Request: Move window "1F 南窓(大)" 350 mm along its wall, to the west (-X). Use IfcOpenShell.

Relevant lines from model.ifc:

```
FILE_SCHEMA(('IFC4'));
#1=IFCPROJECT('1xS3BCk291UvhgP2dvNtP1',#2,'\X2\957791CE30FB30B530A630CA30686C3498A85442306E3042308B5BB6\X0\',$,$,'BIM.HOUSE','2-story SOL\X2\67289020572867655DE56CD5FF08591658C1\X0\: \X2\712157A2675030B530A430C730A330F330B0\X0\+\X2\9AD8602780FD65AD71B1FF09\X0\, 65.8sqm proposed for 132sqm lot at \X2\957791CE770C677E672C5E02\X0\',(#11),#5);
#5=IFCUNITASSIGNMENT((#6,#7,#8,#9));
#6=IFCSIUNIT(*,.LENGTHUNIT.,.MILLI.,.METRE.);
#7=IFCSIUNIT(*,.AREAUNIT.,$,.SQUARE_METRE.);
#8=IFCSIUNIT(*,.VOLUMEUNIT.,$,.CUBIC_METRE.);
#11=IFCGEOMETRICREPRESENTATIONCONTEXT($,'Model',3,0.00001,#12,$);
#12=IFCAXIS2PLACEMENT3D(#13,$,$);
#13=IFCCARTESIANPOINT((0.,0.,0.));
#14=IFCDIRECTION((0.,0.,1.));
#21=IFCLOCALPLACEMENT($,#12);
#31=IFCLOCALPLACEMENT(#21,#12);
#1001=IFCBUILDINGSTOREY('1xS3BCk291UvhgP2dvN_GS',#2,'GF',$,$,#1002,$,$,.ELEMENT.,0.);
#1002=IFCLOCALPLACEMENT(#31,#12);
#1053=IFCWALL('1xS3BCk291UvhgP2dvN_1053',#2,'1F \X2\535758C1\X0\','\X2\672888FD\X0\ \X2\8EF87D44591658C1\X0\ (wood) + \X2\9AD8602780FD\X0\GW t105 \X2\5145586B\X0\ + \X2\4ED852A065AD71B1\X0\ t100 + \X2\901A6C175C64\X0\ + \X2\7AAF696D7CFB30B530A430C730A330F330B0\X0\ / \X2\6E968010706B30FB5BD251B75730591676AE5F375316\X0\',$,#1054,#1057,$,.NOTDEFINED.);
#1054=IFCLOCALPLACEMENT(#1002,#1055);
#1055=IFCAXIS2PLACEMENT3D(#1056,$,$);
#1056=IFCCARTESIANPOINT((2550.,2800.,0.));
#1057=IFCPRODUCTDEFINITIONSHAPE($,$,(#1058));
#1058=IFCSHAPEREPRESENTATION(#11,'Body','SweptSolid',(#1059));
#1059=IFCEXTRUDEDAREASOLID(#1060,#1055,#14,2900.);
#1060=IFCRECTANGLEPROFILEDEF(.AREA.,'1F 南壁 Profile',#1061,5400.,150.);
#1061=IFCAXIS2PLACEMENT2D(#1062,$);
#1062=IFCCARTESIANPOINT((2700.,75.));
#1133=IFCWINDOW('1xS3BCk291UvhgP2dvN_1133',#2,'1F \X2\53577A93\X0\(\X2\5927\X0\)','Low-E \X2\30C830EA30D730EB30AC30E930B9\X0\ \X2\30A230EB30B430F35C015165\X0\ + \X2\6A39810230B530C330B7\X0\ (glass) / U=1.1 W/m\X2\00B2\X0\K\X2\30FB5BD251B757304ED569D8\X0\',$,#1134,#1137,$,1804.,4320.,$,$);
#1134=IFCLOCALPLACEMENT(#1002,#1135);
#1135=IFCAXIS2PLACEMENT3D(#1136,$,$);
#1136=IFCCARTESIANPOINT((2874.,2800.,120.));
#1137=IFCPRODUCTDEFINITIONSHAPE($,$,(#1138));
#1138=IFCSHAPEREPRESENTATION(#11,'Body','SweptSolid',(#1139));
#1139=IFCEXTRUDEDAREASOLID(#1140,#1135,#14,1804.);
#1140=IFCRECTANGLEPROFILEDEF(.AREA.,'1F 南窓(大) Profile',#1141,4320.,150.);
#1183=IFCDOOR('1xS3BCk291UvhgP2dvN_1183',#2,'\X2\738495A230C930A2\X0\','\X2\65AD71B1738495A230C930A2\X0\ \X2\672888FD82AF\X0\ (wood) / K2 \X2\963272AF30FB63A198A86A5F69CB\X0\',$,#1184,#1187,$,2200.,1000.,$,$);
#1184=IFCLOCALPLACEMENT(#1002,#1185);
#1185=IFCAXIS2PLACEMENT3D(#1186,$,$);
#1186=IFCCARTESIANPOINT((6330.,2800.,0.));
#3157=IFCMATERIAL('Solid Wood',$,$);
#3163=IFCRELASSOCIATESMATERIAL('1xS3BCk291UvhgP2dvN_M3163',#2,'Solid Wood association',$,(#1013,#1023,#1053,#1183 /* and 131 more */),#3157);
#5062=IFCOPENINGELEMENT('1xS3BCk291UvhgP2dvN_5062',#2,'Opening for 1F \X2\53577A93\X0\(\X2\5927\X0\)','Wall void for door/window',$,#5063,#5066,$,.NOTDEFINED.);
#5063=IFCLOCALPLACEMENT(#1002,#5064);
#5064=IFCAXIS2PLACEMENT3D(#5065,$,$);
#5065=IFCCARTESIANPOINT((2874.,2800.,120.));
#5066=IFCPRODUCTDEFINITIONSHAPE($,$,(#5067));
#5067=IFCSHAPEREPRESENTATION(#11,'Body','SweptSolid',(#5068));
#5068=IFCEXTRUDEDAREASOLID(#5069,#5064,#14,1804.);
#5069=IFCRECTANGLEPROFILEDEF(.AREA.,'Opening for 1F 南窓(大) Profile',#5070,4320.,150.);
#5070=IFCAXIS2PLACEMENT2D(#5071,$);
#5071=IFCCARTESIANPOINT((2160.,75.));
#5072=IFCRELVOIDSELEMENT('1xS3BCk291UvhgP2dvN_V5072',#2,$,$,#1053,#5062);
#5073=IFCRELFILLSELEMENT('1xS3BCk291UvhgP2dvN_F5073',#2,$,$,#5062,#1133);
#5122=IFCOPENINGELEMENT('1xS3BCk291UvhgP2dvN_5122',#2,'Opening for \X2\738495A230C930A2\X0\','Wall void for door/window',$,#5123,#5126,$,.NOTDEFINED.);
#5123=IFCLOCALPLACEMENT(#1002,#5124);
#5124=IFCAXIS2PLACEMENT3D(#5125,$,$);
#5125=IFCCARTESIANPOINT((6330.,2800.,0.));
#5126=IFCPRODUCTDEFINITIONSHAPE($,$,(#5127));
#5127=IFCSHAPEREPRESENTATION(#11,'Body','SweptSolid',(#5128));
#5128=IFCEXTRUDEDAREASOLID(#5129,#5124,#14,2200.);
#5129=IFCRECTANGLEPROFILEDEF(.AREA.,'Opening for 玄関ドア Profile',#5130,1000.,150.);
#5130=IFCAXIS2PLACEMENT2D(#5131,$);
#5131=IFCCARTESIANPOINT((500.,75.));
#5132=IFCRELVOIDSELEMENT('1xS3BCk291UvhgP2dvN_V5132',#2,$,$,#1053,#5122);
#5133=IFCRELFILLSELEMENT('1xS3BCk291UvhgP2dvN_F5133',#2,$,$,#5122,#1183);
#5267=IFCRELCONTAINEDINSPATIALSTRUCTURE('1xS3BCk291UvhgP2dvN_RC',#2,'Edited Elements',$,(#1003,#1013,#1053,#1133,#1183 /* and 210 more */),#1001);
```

```python
import ifcopenshell
import ifcopenshell.api.geometry
import ifcopenshell.util.placement

model = ifcopenshell.open("model.ifc")

window = model.by_id(1133)
opening = window.FillsVoids[0].RelatingOpeningElement
wall = opening.VoidsElements[0].RelatingBuildingElement

wall_matrix = ifcopenshell.util.placement.get_local_placement(wall.ObjectPlacement)
shift = wall_matrix[:3, 0] * -350.0
before = ifcopenshell.util.placement.get_local_placement(window.ObjectPlacement)[:3, 3].copy()

# The window is not placed relative to its opening, so move both.
for product in (opening, window):
    matrix = ifcopenshell.util.placement.get_local_placement(product.ObjectPlacement)
    matrix[:3, 3] += shift
    ifcopenshell.api.geometry.edit_object_placement(model, product=product, matrix=matrix, is_si=False)

after = ifcopenshell.util.placement.get_local_placement(window.ObjectPlacement)[:3, 3]
print("window moved by", (after - before).round(3) + 0.0)

model.write("model_updated.ifc")
```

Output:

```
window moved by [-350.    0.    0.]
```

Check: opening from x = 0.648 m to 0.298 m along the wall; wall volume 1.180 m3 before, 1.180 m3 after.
